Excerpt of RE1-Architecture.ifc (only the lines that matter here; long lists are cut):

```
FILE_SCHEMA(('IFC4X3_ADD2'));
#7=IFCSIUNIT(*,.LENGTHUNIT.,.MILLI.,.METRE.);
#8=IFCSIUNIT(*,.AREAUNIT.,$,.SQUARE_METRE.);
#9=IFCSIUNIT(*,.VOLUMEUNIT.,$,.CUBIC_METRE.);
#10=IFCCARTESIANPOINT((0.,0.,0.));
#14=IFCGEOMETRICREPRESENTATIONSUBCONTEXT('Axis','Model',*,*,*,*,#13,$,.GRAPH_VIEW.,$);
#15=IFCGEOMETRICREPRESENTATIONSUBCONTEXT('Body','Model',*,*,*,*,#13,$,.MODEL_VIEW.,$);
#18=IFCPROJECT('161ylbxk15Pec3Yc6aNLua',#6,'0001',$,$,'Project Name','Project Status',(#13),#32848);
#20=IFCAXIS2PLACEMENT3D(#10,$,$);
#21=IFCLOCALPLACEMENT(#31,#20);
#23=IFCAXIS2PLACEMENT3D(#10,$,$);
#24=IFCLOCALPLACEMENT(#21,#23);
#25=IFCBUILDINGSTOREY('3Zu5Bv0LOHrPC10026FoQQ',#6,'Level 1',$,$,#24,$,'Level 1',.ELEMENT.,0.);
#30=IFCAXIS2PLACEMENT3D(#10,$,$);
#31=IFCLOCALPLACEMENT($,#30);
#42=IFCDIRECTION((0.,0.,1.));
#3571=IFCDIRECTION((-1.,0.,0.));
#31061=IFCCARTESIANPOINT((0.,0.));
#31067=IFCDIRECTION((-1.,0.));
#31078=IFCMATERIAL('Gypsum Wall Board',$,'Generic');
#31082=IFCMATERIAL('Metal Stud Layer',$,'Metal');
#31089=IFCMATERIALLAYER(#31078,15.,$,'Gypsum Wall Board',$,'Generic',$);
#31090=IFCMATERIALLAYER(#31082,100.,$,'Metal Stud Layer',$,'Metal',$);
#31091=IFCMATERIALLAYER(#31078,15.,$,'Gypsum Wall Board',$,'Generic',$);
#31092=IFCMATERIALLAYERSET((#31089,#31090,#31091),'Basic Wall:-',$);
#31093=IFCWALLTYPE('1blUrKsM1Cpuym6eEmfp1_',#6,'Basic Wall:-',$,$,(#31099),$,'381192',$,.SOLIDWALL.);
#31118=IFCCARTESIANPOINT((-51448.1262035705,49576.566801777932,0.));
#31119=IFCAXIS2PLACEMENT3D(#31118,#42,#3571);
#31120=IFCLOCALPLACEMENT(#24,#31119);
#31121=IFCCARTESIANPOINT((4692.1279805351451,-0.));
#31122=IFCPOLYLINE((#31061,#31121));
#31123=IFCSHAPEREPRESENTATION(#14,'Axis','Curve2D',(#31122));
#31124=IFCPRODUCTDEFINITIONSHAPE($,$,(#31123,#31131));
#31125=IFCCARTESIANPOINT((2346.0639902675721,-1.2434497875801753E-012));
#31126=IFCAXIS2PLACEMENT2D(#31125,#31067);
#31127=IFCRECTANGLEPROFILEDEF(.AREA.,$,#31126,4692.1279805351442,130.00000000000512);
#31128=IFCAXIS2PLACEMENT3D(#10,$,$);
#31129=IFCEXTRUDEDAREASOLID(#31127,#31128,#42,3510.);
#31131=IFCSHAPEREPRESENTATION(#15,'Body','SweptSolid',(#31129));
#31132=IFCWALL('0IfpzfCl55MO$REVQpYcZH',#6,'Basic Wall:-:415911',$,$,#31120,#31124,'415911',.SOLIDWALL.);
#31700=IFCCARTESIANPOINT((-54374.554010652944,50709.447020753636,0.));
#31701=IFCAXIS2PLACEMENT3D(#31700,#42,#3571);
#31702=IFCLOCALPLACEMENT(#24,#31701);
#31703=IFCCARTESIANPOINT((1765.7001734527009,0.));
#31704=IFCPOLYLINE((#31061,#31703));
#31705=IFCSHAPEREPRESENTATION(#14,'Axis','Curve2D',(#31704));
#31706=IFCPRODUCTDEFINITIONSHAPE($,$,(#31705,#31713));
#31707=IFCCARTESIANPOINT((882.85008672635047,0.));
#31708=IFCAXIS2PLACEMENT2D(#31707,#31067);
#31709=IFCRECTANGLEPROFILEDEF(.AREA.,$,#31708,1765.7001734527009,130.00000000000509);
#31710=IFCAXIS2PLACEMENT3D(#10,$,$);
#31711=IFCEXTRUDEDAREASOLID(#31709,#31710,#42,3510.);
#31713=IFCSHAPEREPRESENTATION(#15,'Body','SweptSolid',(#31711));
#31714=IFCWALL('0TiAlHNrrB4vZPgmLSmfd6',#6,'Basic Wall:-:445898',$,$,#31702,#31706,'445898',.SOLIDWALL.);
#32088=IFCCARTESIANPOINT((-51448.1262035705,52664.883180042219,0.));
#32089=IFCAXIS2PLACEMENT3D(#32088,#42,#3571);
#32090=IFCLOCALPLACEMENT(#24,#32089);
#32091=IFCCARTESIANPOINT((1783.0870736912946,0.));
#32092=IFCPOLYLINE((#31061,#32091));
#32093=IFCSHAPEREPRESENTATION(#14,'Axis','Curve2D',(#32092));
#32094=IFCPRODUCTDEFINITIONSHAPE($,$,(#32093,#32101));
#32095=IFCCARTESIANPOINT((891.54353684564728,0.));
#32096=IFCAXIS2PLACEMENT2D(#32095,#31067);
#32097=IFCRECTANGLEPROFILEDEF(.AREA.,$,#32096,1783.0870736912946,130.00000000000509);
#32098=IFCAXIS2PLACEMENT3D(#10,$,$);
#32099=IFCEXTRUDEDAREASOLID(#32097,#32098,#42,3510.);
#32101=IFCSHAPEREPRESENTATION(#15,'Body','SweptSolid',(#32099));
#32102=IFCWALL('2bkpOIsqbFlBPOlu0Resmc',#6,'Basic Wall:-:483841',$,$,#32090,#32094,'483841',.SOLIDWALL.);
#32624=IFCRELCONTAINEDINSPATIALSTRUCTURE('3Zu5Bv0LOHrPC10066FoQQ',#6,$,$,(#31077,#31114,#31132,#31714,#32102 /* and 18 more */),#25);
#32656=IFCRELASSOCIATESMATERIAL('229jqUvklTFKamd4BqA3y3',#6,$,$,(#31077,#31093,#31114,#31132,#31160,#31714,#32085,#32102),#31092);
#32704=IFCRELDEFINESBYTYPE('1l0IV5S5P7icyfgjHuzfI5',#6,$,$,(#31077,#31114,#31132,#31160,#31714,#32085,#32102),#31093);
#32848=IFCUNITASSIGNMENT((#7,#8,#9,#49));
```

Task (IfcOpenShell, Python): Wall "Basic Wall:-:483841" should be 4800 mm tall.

```python
import ifcopenshell
import ifcopenshell.geom
import ifcopenshell.util.representation
import ifcopenshell.util.shape

model = ifcopenshell.open("RE1-Architecture.ifc")
settings = ifcopenshell.geom.settings()


def volume(element):
    """Net volume in cubic metres, openings subtracted."""
    shape = ifcopenshell.geom.create_shape(settings, element)
    return ifcopenshell.util.shape.get_volume(shape.geometry)


wall = model.by_guid("2bkpOIsqbFlBPOlu0Resmc")
before = volume(wall)

body = ifcopenshell.util.representation.get_representation(wall, "Model", "Body")
solid = body.Items[0]
old_height = solid.Depth
solid.Depth = 4800.0
after = volume(wall)

print(f"height {old_height:g} -> {solid.Depth:g}, volume {before:.3f} -> {after:.3f} m3")

model.write("RE1-Architecture_edited.ifc")
```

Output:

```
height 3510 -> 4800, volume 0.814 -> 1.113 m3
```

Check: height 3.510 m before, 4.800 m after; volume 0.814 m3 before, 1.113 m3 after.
